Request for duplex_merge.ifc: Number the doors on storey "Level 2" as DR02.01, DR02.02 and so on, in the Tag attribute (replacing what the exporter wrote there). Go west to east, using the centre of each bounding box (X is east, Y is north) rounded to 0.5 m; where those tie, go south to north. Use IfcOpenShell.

First a look at what the model holds.

```python
import ifcopenshell
import ifcopenshell.util.element
import ifcopenshell.util.placement

model = ifcopenshell.open("duplex_merge.ifc")
print(model.schema)
storey = next(s for s in model.by_type("IfcBuildingStorey") if s.Name == "Level 2")
doors = [e for e in ifcopenshell.util.element.get_decomposition(storey) if e.is_a("IfcDoor")]
for e in sorted(doors, key=lambda e: e.id()):
    origin = ifcopenshell.util.placement.get_local_placement(e.ObjectPlacement)[:3, 3]
    print(e.id(), e.Tag, e.Name, origin.round(2) + 0.0, sep=" | ")
```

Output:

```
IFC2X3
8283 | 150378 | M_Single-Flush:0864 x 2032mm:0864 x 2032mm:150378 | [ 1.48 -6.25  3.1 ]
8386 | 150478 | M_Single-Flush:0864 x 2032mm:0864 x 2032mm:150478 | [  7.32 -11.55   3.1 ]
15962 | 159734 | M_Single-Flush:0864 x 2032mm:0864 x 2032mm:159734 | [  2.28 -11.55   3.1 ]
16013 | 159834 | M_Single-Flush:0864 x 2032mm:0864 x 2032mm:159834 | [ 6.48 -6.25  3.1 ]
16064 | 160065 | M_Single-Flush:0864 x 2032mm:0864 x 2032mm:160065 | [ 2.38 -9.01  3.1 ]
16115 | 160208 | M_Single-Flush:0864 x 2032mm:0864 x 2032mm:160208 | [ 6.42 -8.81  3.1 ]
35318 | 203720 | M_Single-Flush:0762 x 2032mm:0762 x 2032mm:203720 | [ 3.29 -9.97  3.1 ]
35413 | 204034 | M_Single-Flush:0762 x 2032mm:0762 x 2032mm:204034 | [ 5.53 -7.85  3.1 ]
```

```python
import ifcopenshell
import ifcopenshell.geom
import ifcopenshell.util.element
import ifcopenshell.util.shape

model = ifcopenshell.open("duplex_merge.ifc")
settings = ifcopenshell.geom.settings()
settings.set("use-world-coords", True)


def centre(element):
    shape = ifcopenshell.geom.create_shape(settings, element)
    return ifcopenshell.util.shape.get_bbox_centroid(shape.geometry)


storey = next(s for s in model.by_type("IfcBuildingStorey") if s.Name == "Level 2")
doors = [e for e in ifcopenshell.util.element.get_decomposition(storey) if e.is_a("IfcDoor")]

# Insertion points can sit at a corner or the storey origin, so sort by the geometry (in metres).
centres = {e: centre(e) for e in doors}
doors.sort(key=lambda e: (round(centres[e][0] / 0.5), centres[e][1]))

for i, e in enumerate(doors, start=1):
    number = f"DR02.{i:02d}"
    e.Tag = number
    print(e.id(), number)

model.write("duplex_merge_rev.ifc")
```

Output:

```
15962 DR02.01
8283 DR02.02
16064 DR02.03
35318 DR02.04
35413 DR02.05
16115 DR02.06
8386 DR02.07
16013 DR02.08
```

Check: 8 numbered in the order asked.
